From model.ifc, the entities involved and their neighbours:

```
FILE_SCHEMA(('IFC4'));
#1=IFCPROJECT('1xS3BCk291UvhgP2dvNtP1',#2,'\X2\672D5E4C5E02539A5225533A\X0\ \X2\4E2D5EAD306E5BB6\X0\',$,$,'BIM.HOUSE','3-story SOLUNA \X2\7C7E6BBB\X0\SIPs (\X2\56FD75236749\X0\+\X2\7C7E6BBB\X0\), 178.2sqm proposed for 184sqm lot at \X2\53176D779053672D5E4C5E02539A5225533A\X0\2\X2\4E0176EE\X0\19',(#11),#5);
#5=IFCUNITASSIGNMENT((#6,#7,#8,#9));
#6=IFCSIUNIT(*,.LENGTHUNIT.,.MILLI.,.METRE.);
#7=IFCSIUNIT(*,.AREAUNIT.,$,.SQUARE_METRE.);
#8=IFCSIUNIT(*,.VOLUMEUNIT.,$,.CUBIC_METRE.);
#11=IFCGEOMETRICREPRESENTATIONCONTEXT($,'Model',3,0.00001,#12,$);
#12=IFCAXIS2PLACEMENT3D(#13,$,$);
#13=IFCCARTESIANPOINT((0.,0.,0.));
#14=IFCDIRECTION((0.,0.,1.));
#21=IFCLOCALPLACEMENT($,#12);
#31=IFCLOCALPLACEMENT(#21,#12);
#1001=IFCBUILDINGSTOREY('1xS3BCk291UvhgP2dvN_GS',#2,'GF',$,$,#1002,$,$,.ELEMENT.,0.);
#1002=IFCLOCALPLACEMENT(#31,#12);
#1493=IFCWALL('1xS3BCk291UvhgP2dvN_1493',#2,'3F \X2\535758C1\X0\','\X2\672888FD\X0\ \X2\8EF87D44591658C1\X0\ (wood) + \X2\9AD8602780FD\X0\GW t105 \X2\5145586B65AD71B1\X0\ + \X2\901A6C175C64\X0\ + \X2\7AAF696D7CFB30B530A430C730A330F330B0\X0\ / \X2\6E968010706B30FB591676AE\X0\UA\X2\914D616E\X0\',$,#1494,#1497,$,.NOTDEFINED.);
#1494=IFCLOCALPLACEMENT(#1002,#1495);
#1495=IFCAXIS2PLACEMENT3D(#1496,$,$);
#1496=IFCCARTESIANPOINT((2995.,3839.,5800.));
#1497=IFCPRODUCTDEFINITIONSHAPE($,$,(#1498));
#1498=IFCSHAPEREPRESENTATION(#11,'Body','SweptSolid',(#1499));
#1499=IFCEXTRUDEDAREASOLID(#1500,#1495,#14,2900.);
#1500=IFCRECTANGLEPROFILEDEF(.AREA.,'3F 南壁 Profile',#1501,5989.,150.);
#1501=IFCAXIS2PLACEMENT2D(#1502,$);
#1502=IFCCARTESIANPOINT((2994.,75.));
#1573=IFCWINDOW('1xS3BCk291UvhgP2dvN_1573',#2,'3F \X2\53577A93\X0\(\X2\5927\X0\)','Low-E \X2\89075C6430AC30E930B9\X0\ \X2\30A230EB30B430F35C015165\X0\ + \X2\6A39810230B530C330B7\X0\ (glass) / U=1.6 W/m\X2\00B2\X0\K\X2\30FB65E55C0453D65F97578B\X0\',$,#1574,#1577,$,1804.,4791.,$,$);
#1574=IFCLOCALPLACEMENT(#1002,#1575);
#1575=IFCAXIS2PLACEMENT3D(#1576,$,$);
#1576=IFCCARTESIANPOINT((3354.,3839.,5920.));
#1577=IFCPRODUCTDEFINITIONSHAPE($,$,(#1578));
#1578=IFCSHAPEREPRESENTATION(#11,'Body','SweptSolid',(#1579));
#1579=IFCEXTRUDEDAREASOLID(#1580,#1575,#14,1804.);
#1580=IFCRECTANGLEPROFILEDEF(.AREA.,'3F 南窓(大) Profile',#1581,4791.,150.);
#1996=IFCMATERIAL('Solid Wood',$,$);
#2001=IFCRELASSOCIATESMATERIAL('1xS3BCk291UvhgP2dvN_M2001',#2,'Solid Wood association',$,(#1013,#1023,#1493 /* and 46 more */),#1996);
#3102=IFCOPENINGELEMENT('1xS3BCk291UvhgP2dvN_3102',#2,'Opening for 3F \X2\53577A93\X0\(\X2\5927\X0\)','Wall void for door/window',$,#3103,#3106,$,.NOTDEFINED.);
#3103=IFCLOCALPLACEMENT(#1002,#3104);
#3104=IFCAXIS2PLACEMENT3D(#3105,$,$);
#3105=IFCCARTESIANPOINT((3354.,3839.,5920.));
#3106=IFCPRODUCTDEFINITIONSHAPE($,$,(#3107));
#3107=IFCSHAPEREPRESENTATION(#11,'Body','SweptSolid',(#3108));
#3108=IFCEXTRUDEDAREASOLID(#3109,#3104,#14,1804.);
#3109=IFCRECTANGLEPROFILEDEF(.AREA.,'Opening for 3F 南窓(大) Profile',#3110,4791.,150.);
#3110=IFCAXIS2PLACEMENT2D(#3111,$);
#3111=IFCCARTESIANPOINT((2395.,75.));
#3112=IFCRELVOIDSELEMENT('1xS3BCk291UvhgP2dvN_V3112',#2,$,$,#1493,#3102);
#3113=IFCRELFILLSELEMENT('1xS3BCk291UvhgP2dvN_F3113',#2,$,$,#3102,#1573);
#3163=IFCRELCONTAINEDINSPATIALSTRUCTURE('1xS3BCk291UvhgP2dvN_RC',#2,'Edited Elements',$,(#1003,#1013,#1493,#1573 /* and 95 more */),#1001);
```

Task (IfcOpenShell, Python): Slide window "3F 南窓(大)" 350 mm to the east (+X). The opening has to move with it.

```python
import ifcopenshell
import ifcopenshell.api.geometry
import ifcopenshell.util.placement
import ifcopenshell.util.unit

model = ifcopenshell.open("model.ifc")
unit_scale = ifcopenshell.util.unit.calculate_unit_scale(model)

window = model.by_id(1573)
opening = window.FillsVoids[0].RelatingOpeningElement
wall = opening.VoidsElements[0].RelatingBuildingElement

wall_matrix = ifcopenshell.util.placement.get_local_placement(wall.ObjectPlacement)
shift = wall_matrix[:3, 0] * 0.35 / unit_scale
before = ifcopenshell.util.placement.get_local_placement(window.ObjectPlacement)[:3, 3].copy()

# The window is not placed relative to its opening, so move both.
for product in (opening, window):
    matrix = ifcopenshell.util.placement.get_local_placement(product.ObjectPlacement)
    matrix[:3, 3] += shift
    ifcopenshell.api.geometry.edit_object_placement(model, product=product, matrix=matrix, is_si=False)

after = ifcopenshell.util.placement.get_local_placement(window.ObjectPlacement)[:3, 3]
print("window moved by", (after - before).round(3) + 0.0)

model.write("model_updated.ifc")
```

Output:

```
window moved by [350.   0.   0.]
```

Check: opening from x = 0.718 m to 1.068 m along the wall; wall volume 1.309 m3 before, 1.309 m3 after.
